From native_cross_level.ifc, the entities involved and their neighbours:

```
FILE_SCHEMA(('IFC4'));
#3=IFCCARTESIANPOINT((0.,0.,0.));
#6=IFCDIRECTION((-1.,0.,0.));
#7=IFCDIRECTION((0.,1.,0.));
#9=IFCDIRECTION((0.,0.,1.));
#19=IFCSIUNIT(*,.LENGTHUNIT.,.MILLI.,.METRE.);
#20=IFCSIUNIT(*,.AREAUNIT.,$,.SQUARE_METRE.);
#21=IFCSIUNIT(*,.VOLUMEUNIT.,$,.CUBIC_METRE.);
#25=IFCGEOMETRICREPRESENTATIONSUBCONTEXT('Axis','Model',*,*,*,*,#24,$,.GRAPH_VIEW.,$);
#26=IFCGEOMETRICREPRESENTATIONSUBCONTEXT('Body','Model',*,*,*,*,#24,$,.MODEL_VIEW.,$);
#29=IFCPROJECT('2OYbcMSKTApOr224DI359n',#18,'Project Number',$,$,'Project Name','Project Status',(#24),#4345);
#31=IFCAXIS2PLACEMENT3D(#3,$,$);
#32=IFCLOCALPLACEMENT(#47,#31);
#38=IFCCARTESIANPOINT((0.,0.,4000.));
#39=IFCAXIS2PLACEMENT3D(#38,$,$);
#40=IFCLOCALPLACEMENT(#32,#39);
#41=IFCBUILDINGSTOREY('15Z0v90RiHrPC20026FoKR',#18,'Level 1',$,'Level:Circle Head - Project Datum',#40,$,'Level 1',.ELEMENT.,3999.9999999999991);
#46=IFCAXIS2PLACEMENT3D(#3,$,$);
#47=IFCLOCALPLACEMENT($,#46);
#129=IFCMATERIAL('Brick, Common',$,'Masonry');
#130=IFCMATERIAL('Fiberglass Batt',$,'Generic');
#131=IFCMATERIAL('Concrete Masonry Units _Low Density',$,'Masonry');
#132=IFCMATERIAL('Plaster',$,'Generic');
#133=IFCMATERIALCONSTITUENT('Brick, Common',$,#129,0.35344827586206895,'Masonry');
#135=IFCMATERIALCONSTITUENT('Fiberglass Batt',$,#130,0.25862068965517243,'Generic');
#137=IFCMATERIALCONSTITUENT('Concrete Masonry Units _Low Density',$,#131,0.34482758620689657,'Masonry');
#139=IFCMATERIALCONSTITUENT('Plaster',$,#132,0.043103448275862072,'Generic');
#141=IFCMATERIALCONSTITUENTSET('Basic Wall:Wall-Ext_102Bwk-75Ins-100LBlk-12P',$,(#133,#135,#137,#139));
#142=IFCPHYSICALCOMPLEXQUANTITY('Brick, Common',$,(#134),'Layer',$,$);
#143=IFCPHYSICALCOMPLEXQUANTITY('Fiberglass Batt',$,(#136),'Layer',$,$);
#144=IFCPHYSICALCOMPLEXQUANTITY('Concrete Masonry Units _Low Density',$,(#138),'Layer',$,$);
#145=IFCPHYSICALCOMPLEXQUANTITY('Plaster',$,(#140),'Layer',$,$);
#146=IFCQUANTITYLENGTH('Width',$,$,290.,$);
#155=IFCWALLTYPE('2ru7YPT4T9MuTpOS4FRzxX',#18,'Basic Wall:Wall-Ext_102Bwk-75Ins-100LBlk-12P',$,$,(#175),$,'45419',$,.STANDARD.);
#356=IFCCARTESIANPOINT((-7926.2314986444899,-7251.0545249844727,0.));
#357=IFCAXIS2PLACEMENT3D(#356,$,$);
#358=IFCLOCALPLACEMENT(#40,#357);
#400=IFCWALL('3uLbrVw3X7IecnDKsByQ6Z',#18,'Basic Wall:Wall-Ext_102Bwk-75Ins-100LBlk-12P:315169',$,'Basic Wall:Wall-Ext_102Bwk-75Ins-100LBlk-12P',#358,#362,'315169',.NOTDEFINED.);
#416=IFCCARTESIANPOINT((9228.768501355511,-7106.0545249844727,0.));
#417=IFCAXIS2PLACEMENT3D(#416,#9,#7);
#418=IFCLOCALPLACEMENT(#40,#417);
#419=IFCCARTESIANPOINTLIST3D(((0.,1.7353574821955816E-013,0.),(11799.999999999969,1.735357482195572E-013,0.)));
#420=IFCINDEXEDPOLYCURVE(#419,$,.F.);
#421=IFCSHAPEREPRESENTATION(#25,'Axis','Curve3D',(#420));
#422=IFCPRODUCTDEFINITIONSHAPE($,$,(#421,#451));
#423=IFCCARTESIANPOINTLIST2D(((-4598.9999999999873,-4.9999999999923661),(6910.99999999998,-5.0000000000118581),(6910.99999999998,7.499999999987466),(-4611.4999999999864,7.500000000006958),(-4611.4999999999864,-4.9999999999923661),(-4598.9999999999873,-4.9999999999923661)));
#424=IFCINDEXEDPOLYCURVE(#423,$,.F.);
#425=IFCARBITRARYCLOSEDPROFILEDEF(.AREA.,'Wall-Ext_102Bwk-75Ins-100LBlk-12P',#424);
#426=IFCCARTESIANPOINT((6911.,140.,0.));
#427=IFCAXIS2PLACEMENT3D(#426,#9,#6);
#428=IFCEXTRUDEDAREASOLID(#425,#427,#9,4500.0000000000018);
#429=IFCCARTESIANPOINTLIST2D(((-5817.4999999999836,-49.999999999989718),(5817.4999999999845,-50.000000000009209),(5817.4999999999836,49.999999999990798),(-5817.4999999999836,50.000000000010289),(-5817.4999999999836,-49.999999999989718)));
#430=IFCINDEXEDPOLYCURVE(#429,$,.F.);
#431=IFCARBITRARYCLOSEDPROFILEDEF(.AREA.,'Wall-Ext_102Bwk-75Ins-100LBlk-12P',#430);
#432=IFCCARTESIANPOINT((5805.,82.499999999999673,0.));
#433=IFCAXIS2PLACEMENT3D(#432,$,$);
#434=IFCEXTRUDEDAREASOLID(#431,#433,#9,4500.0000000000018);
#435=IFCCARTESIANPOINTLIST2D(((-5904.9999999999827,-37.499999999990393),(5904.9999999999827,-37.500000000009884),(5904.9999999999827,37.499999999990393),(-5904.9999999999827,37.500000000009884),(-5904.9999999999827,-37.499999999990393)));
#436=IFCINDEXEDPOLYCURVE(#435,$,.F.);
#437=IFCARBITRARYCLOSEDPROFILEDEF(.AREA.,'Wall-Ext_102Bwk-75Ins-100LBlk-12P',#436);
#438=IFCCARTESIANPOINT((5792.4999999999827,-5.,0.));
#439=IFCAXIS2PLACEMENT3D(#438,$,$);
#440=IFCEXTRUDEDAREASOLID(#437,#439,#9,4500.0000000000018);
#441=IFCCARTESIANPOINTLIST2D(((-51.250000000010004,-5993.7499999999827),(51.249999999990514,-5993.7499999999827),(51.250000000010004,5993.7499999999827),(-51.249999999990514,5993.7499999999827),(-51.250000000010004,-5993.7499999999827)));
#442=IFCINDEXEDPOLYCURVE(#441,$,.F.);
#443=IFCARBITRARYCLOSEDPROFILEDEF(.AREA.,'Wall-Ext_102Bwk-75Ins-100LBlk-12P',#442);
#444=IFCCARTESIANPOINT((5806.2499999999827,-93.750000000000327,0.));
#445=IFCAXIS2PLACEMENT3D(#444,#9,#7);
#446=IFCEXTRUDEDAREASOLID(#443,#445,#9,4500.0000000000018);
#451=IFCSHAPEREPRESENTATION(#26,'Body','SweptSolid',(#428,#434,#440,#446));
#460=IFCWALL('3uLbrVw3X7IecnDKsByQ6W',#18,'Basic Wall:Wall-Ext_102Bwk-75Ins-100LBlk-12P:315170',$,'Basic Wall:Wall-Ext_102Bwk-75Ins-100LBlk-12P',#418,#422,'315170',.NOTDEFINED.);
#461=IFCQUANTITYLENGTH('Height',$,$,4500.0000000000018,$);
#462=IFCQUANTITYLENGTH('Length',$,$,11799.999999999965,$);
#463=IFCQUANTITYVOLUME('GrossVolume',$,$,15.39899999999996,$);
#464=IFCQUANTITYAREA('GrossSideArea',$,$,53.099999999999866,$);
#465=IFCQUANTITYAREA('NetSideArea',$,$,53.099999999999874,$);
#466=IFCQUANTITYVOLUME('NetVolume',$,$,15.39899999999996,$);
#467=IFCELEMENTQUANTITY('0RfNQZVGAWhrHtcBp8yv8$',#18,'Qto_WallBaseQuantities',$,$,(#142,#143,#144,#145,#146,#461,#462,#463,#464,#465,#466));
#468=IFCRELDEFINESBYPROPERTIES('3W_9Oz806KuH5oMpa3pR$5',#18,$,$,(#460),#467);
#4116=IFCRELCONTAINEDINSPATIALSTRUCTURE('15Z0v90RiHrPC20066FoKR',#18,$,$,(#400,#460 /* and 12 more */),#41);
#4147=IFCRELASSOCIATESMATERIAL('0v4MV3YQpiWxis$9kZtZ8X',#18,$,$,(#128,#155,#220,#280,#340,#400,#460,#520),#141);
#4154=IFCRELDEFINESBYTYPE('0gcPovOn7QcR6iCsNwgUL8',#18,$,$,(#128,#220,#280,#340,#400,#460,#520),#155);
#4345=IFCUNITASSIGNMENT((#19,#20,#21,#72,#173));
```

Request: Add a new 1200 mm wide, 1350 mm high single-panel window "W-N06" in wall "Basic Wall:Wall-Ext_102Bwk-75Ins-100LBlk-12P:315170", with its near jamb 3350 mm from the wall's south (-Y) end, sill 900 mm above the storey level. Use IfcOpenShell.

```python
import numpy as np
import ifcopenshell
import ifcopenshell.api.feature
import ifcopenshell.api.geometry
import ifcopenshell.api.pset
import ifcopenshell.api.root
import ifcopenshell.api.spatial
import ifcopenshell.geom
import ifcopenshell.util.element
import ifcopenshell.util.placement
import ifcopenshell.util.representation
import ifcopenshell.util.shape
import ifcopenshell.util.unit

model = ifcopenshell.open("native_cross_level.ifc")
unit_scale = ifcopenshell.util.unit.calculate_unit_scale(model)
area_scale = ifcopenshell.util.unit.calculate_unit_scale(model, "AREAUNIT")
volume_scale = ifcopenshell.util.unit.calculate_unit_scale(model, "VOLUMEUNIT")
settings = ifcopenshell.geom.settings()


def volume(element):
    """Net volume in cubic metres, openings subtracted."""
    shape = ifcopenshell.geom.create_shape(settings, element)
    return ifcopenshell.util.shape.get_volume(shape.geometry)


wall = model.by_guid("3uLbrVw3X7IecnDKsByQ6W")
storey = ifcopenshell.util.element.get_container(wall, ifc_class="IfcBuildingStorey")
context = ifcopenshell.util.representation.get_context(model, "Model", "Body", "MODEL_VIEW")
before = volume(wall)

width, height, from_end, sill = 1.2, 1.35, 3.35, 0.9  # metres

# The wall runs along its own X axis, and the end named is its -X end.
wall_shape = ifcopenshell.geom.create_shape(settings, wall)
x, y, z = ifcopenshell.util.shape.get_vertices(wall_shape.geometry).T
start = x.min() + from_end
face, thickness = float(y.min()), float(y.max() - y.min())
wall_matrix = ifcopenshell.util.placement.get_local_placement(wall.ObjectPlacement)
level = ifcopenshell.util.placement.get_local_placement(storey.ObjectPlacement)[2, 3]


def in_wall(x, y):
    """Placement at x, y metres in the wall's axes, at sill height."""
    matrix = wall_matrix.copy()
    matrix[:, 3] = wall_matrix @ np.array([x / unit_scale, y / unit_scale, 0.0, 1.0])
    matrix[2, 3] = level + sill / unit_scale
    return matrix


# Opening: a box that overshoots both wall faces by 50 mm.
opening = ifcopenshell.api.root.create_entity(model, ifc_class="IfcOpeningElement", predefined_type="OPENING")
box = ifcopenshell.api.geometry.add_wall_representation(
    model, context=context, length=width, height=height, thickness=thickness + 0.1
)
ifcopenshell.api.geometry.assign_representation(model, product=opening, representation=box)
ifcopenshell.api.geometry.edit_object_placement(model, product=opening, matrix=in_wall(start, face - 0.05), is_si=False)
ifcopenshell.api.feature.add_feature(model, feature=opening, element=wall)

window = ifcopenshell.api.root.create_entity(model, ifc_class="IfcWindow", name="W-N06", predefined_type="WINDOW")
window.OverallWidth, window.OverallHeight = width / unit_scale, height / unit_scale
window.PartitioningType = "SINGLE_PANEL"
body = ifcopenshell.api.geometry.add_window_representation(
    model,
    context=context,
    overall_width=window.OverallWidth,
    overall_height=window.OverallHeight,
    partition_type="SINGLE_PANEL",
)
ifcopenshell.api.geometry.assign_representation(model, product=window, representation=body)
ifcopenshell.api.spatial.assign_container(model, products=[window], relating_structure=storey)
ifcopenshell.api.feature.add_filling(model, opening=opening, element=window)

# Centre the window in the wall's thickness.
ifcopenshell.api.geometry.edit_object_placement(model, product=window, matrix=in_wall(start, face), is_si=False)
window_shape = ifcopenshell.geom.create_shape(settings, window)
depth = ifcopenshell.util.shape.get_vertices(window_shape.geometry)[:, 1]
offset = face + thickness / 2 - (depth.min() + depth.max()) / 2
ifcopenshell.api.geometry.edit_object_placement(model, product=window, matrix=in_wall(start, offset), is_si=False)

after = volume(wall)

# Update the wall's stored quantities.
qto = model.by_id(ifcopenshell.util.element.get_pset(wall, "Qto_WallBaseQuantities", should_inherit=False)["id"])
ifcopenshell.api.pset.edit_qto(model, qto=qto, properties={
    "NetSideArea": after / thickness / area_scale,
    "NetVolume": after / volume_scale,
})

print(f"wall volume {before:.3f} -> {after:.3f} m3")

model.write("native_cross_level_updated.ifc")
```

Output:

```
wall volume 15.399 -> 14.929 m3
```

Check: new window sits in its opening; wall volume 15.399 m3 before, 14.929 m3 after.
